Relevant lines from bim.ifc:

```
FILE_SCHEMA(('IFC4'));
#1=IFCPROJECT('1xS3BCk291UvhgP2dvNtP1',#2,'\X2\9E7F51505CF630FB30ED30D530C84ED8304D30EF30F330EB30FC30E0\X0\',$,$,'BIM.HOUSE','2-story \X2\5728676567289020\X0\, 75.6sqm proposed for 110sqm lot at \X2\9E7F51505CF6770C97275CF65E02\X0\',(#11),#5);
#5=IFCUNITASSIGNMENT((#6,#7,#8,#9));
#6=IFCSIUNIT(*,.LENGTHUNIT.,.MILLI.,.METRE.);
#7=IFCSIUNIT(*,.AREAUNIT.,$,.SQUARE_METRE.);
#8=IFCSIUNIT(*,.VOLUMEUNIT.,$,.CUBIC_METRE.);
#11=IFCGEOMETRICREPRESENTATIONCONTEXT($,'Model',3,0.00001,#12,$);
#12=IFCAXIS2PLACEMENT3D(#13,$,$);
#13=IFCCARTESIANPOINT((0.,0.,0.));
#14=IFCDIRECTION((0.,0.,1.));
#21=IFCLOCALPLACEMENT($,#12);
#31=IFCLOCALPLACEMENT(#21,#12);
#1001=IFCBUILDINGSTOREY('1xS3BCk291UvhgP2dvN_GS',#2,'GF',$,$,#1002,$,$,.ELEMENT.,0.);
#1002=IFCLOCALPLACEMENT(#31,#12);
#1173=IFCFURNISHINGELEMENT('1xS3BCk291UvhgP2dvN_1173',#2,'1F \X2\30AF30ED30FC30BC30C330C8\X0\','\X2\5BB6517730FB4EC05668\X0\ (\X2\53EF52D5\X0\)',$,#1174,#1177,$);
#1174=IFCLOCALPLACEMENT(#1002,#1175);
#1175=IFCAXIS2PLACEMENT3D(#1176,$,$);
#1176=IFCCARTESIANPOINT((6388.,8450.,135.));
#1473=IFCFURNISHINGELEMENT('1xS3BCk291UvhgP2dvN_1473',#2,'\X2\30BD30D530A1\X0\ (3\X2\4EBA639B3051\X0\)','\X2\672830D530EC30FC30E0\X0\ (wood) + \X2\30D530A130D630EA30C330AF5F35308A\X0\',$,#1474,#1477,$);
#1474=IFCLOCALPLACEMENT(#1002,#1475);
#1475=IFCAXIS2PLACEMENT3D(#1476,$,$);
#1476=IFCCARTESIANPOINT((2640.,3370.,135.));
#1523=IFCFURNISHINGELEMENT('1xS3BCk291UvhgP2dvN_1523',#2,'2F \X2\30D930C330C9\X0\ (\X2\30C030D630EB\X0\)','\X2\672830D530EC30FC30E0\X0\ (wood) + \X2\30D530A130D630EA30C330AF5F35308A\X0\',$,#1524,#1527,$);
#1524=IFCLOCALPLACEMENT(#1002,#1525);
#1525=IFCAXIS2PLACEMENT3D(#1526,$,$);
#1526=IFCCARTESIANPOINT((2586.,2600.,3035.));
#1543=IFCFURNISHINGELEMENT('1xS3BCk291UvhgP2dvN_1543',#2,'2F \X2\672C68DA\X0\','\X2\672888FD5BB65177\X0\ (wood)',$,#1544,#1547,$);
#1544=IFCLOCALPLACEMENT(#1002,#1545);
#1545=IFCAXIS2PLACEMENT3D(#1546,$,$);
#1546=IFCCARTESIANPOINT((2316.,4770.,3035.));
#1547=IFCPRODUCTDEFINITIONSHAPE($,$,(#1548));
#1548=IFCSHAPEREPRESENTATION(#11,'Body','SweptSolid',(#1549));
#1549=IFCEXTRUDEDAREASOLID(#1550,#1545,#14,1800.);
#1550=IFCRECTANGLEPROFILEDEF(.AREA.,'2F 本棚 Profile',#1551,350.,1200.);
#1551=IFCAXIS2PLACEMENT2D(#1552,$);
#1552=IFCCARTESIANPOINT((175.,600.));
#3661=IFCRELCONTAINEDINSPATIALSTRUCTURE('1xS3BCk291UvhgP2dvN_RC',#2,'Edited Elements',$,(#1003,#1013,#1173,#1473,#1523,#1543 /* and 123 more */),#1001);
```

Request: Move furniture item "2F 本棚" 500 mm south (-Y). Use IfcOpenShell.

```python
import ifcopenshell
import ifcopenshell.api.geometry
import ifcopenshell.util.placement
import ifcopenshell.util.unit

model = ifcopenshell.open("bim.ifc")
unit_scale = ifcopenshell.util.unit.calculate_unit_scale(model)

item = model.by_guid("1xS3BCk291UvhgP2dvN_1543")
matrix = ifcopenshell.util.placement.get_local_placement(item.ObjectPlacement)
matrix[1, 3] -= 0.5 / unit_scale
ifcopenshell.api.geometry.edit_object_placement(model, product=item, matrix=matrix, is_si=False)

print(ifcopenshell.util.placement.get_local_placement(item.ObjectPlacement).round(3) + 0.0)

model.write("bim_v2.ifc")
```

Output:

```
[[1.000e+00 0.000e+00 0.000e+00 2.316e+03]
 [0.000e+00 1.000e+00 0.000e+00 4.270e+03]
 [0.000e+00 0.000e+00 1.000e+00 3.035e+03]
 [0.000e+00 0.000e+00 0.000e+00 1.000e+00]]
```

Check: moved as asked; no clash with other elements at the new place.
